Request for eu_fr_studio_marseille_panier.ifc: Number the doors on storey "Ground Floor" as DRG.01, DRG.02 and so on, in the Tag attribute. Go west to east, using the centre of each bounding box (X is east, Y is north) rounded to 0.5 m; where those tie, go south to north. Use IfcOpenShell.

First a look at what the model holds.

```python
import ifcopenshell
import ifcopenshell.util.element
import ifcopenshell.util.placement

model = ifcopenshell.open("eu_fr_studio_marseille_panier.ifc")
print(model.schema)
storey = next(s for s in model.by_type("IfcBuildingStorey") if s.Name == "Ground Floor")
doors = [e for e in ifcopenshell.util.element.get_decomposition(storey) if e.is_a("IfcDoor")]
for e in sorted(doors, key=lambda e: e.id()):
    origin = ifcopenshell.util.placement.get_local_placement(e.ObjectPlacement)[:3, 3]
    print(e.id(), e.Tag, e.Name, origin.round(2) + 0.0, sep=" | ")
```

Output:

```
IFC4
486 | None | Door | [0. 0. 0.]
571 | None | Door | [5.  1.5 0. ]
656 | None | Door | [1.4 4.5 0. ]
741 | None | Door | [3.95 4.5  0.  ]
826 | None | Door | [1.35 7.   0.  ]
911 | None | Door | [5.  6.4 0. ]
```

```python
import ifcopenshell
import ifcopenshell.geom
import ifcopenshell.util.element
import ifcopenshell.util.shape

model = ifcopenshell.open("eu_fr_studio_marseille_panier.ifc")
settings = ifcopenshell.geom.settings()
settings.set("use-world-coords", True)


def centre(element):
    shape = ifcopenshell.geom.create_shape(settings, element)
    return ifcopenshell.util.shape.get_bbox_centroid(shape.geometry)


storey = next(s for s in model.by_type("IfcBuildingStorey") if s.Name == "Ground Floor")
doors = [e for e in ifcopenshell.util.element.get_decomposition(storey) if e.is_a("IfcDoor")]

# Insertion points can sit at a corner or the storey origin, so sort by the geometry (in metres).
centres = {e: centre(e) for e in doors}
doors.sort(key=lambda e: (round(centres[e][0] / 0.5), centres[e][1]))

for i, e in enumerate(doors, start=1):
    number = f"DRG.{i:02d}"
    e.Tag = number
    print(e.id(), number)

model.write("eu_fr_studio_marseille_panier_rev.ifc")
```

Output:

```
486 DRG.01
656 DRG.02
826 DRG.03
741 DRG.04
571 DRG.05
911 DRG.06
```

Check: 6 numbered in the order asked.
